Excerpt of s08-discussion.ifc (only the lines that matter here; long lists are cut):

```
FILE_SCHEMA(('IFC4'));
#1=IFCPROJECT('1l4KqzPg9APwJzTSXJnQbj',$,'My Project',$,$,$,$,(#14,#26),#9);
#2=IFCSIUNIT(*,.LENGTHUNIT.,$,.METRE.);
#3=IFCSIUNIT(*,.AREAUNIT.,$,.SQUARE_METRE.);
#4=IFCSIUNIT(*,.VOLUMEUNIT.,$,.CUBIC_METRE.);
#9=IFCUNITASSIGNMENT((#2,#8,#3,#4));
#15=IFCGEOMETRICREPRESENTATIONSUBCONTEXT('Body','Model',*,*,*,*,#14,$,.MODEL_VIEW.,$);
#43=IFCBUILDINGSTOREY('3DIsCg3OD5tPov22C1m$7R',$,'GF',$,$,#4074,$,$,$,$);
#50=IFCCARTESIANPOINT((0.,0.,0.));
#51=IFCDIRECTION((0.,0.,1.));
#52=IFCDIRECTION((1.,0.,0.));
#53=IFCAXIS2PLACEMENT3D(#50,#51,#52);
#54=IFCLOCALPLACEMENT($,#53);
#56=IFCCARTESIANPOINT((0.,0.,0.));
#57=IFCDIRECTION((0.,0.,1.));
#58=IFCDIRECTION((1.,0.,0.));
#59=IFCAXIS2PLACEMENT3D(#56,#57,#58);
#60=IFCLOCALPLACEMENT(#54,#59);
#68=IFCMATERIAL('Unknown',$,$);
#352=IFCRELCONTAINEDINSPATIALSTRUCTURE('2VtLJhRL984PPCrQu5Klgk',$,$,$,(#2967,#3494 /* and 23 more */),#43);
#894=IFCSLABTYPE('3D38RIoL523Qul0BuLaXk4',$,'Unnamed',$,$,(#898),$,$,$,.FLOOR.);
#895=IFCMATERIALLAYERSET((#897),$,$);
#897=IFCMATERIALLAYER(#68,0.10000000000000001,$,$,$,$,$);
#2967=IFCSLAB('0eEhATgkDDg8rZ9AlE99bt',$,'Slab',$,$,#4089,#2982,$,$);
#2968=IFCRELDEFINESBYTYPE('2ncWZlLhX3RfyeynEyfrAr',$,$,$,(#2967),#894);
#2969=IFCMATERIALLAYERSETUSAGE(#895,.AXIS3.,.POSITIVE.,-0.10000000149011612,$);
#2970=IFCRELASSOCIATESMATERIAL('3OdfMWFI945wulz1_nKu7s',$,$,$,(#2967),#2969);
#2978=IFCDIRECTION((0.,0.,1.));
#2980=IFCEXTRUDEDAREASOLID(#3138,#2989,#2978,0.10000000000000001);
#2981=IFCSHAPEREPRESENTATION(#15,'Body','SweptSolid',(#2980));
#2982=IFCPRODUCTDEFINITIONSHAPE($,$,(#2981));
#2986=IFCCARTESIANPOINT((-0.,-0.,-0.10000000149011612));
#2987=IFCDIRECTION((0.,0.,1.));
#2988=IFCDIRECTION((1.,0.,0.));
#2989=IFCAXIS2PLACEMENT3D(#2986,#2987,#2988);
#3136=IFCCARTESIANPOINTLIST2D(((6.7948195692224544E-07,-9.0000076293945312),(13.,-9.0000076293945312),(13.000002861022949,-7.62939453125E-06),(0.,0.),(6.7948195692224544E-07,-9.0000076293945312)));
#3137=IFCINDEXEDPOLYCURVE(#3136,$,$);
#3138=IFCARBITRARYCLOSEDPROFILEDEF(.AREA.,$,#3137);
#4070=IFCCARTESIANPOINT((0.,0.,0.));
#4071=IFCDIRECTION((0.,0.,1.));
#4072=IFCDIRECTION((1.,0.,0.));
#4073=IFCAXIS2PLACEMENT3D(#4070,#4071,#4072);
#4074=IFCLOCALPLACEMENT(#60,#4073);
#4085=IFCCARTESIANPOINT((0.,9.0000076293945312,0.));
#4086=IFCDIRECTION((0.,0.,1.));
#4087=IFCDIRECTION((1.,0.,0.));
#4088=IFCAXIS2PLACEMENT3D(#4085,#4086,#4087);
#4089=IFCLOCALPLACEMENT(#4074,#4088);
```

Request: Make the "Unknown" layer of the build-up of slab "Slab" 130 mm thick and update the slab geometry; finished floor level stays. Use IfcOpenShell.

```python
import ifcopenshell
import ifcopenshell.util.element
import ifcopenshell.util.representation

model = ifcopenshell.open("s08-discussion.ifc")

layer_set = model.by_id(895)
layer = next(l for l in layer_set.MaterialLayers if l.Material and l.Material.Name == "Unknown")
change = 0.13 - layer.LayerThickness
layer.LayerThickness += change

# Geometry does not follow the layer set by itself.
slabs = [e for e in ifcopenshell.util.element.get_elements_by_material(model, layer_set) if e.is_a("IfcSlab")]
for slab in sorted(slabs, key=lambda e: e.id()):
    body = ifcopenshell.util.representation.get_representation(slab, "Model", "Body")
    solid = body.Items[0]
    old_depth = solid.Depth
    solid.Depth += change
    # Extruded upwards: lower the start of the extrusion so the top stays.
    x, y, z = solid.Position.Location.Coordinates
    solid.Position.Location = model.createIfcCartesianPoint((x, y, z - change))
    print(slab.id(), f"{old_depth:g} -> {solid.Depth:g}")

# The layers are counted up from the underside, which has moved.
for usage in {ifcopenshell.util.element.get_material(slab) for slab in slabs}:
    usage.OffsetFromReferenceLine -= change

model.write("s08-discussion-out.ifc")
```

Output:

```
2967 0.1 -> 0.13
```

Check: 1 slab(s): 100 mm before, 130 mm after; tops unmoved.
